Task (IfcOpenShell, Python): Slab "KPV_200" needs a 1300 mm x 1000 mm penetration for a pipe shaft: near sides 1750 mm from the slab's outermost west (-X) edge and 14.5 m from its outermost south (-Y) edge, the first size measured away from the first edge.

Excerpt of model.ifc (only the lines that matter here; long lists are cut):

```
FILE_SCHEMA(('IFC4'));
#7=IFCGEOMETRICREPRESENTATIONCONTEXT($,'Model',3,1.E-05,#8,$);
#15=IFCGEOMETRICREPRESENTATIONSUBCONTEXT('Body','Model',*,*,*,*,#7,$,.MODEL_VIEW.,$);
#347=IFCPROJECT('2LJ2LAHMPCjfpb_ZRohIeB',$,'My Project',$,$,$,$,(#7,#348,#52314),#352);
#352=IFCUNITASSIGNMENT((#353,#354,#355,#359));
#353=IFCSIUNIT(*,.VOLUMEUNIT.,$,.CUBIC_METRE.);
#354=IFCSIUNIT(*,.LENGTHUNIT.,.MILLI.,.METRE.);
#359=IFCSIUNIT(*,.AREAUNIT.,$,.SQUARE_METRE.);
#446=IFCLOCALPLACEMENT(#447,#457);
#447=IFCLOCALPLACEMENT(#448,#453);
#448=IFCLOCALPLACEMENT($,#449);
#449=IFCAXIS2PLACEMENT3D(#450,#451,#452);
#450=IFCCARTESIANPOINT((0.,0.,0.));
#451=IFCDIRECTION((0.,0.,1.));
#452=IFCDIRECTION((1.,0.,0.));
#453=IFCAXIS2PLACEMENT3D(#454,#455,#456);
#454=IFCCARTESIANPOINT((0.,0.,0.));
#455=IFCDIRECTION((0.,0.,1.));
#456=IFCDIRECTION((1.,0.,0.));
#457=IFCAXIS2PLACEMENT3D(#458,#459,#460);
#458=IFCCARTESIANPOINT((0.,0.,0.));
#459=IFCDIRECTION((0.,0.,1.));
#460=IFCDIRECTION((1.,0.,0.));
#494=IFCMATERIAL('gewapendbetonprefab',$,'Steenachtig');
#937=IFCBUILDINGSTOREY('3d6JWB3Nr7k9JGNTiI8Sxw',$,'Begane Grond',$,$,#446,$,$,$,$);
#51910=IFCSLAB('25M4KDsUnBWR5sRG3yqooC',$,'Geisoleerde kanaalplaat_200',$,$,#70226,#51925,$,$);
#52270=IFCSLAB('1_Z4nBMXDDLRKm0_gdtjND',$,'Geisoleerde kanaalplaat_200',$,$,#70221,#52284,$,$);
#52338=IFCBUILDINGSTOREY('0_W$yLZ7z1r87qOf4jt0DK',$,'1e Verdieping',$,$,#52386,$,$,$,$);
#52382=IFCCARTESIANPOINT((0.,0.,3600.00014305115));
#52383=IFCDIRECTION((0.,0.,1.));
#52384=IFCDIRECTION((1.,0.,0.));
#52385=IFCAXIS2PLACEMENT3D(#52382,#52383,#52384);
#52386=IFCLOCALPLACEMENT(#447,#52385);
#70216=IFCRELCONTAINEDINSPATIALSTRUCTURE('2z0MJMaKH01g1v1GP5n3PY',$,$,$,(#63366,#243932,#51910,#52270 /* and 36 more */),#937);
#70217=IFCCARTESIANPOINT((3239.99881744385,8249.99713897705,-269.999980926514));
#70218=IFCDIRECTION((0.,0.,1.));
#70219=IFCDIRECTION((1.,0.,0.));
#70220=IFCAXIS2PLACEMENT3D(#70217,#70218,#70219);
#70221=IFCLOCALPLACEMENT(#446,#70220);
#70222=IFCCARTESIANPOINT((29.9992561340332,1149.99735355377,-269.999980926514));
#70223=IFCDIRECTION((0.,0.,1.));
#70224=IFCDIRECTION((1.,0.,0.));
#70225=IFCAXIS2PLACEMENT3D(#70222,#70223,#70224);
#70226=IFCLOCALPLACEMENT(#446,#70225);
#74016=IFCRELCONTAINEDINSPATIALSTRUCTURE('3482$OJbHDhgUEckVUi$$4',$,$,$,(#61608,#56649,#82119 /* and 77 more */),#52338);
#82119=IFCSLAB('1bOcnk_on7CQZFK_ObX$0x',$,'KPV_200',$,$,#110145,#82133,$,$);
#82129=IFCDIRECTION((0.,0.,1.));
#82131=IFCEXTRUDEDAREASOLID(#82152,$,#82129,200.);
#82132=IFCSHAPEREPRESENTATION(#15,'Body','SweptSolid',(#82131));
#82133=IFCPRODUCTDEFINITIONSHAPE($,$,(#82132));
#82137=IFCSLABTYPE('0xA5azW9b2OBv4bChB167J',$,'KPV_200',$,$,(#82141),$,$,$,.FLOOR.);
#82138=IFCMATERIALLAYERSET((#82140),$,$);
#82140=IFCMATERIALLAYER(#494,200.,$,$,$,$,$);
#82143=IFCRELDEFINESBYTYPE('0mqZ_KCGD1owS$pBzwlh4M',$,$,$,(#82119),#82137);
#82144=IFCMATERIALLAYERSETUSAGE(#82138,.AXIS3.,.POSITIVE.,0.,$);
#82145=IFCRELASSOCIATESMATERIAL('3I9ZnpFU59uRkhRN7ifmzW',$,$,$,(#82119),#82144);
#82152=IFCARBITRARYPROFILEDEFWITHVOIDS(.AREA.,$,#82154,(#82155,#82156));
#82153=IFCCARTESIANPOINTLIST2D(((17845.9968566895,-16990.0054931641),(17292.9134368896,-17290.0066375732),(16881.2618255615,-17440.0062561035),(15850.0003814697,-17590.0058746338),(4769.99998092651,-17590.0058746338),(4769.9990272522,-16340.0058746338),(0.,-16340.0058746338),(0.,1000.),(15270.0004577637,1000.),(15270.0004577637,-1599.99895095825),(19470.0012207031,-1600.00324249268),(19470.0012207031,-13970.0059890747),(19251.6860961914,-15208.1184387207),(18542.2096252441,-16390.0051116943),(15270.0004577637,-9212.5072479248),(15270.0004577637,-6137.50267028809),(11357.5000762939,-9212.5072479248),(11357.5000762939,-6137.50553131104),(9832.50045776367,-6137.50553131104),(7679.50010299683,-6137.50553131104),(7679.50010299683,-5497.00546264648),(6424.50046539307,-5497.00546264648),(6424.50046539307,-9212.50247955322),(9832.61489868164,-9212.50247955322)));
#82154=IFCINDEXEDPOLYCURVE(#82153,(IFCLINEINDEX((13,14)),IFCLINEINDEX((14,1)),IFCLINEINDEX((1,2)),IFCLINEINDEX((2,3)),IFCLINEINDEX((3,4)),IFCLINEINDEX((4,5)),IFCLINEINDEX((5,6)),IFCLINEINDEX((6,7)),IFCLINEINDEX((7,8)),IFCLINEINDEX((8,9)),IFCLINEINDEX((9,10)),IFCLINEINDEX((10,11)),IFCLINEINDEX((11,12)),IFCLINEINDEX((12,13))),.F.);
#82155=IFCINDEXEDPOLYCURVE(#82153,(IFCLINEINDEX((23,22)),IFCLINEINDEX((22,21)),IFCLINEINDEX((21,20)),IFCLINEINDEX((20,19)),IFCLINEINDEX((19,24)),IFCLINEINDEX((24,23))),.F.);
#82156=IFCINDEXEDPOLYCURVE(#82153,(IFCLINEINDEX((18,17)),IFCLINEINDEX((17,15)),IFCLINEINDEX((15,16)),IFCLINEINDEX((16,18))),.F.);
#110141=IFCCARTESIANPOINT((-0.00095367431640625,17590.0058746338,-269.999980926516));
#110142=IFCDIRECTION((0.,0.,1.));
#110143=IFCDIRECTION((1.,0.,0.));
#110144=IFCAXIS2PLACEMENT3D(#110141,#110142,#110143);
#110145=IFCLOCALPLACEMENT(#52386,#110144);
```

```python
import numpy as np
import ifcopenshell
import ifcopenshell.api.feature
import ifcopenshell.api.geometry
import ifcopenshell.api.root
import ifcopenshell.geom
import ifcopenshell.util.placement
import ifcopenshell.util.representation
import ifcopenshell.util.shape
import ifcopenshell.util.unit

model = ifcopenshell.open("model.ifc")
unit_scale = ifcopenshell.util.unit.calculate_unit_scale(model)
settings = ifcopenshell.geom.settings()


def volume(element):
    """Net volume in cubic metres, openings subtracted."""
    shape = ifcopenshell.geom.create_shape(settings, element)
    return ifcopenshell.util.shape.get_volume(shape.geometry)


slab = model.by_guid("1bOcnk_on7CQZFK_ObX$0x")
before = volume(slab)

# Extent in the slab's own axes, in metres. The edges named are its -X and -Y sides.
slab_shape = ifcopenshell.geom.create_shape(settings, slab)
vertices = ifcopenshell.util.shape.get_vertices(slab_shape.geometry)
x_min, y_min, bottom = vertices.min(axis=0)
top = vertices[:, 2].max()

opening = ifcopenshell.api.root.create_entity(model, ifc_class="IfcOpeningElement", name="Pipe shaft opening", predefined_type="OPENING")
context = ifcopenshell.util.representation.get_context(model, "Model", "Body", "MODEL_VIEW")
width, depth = 1.3, 1
outline = [(0.0, 0.0), (width, 0.0), (width, depth), (0.0, depth), (0.0, 0.0)]
# Overshoot both faces by 50 mm so the cut is clean.
shape = ifcopenshell.api.geometry.add_slab_representation(
    model, context=context, depth=top - bottom + 0.1, polyline=outline
)
ifcopenshell.api.geometry.assign_representation(model, product=opening, representation=shape)

matrix = ifcopenshell.util.placement.get_local_placement(slab.ObjectPlacement)
matrix[:, 3] = matrix @ np.append(np.array([x_min + 1.75, y_min + 14.5, bottom - 0.05]) / unit_scale, 1.0)
ifcopenshell.api.geometry.edit_object_placement(model, product=opening, matrix=matrix, is_si=False)
ifcopenshell.api.feature.add_feature(model, feature=opening, element=slab)

after = volume(slab)

print(f"slab volume {before:.3f} -> {after:.3f} m3")

model.write("model_edited.ifc")
```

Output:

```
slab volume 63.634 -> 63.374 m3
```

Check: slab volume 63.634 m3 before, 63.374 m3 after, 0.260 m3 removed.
